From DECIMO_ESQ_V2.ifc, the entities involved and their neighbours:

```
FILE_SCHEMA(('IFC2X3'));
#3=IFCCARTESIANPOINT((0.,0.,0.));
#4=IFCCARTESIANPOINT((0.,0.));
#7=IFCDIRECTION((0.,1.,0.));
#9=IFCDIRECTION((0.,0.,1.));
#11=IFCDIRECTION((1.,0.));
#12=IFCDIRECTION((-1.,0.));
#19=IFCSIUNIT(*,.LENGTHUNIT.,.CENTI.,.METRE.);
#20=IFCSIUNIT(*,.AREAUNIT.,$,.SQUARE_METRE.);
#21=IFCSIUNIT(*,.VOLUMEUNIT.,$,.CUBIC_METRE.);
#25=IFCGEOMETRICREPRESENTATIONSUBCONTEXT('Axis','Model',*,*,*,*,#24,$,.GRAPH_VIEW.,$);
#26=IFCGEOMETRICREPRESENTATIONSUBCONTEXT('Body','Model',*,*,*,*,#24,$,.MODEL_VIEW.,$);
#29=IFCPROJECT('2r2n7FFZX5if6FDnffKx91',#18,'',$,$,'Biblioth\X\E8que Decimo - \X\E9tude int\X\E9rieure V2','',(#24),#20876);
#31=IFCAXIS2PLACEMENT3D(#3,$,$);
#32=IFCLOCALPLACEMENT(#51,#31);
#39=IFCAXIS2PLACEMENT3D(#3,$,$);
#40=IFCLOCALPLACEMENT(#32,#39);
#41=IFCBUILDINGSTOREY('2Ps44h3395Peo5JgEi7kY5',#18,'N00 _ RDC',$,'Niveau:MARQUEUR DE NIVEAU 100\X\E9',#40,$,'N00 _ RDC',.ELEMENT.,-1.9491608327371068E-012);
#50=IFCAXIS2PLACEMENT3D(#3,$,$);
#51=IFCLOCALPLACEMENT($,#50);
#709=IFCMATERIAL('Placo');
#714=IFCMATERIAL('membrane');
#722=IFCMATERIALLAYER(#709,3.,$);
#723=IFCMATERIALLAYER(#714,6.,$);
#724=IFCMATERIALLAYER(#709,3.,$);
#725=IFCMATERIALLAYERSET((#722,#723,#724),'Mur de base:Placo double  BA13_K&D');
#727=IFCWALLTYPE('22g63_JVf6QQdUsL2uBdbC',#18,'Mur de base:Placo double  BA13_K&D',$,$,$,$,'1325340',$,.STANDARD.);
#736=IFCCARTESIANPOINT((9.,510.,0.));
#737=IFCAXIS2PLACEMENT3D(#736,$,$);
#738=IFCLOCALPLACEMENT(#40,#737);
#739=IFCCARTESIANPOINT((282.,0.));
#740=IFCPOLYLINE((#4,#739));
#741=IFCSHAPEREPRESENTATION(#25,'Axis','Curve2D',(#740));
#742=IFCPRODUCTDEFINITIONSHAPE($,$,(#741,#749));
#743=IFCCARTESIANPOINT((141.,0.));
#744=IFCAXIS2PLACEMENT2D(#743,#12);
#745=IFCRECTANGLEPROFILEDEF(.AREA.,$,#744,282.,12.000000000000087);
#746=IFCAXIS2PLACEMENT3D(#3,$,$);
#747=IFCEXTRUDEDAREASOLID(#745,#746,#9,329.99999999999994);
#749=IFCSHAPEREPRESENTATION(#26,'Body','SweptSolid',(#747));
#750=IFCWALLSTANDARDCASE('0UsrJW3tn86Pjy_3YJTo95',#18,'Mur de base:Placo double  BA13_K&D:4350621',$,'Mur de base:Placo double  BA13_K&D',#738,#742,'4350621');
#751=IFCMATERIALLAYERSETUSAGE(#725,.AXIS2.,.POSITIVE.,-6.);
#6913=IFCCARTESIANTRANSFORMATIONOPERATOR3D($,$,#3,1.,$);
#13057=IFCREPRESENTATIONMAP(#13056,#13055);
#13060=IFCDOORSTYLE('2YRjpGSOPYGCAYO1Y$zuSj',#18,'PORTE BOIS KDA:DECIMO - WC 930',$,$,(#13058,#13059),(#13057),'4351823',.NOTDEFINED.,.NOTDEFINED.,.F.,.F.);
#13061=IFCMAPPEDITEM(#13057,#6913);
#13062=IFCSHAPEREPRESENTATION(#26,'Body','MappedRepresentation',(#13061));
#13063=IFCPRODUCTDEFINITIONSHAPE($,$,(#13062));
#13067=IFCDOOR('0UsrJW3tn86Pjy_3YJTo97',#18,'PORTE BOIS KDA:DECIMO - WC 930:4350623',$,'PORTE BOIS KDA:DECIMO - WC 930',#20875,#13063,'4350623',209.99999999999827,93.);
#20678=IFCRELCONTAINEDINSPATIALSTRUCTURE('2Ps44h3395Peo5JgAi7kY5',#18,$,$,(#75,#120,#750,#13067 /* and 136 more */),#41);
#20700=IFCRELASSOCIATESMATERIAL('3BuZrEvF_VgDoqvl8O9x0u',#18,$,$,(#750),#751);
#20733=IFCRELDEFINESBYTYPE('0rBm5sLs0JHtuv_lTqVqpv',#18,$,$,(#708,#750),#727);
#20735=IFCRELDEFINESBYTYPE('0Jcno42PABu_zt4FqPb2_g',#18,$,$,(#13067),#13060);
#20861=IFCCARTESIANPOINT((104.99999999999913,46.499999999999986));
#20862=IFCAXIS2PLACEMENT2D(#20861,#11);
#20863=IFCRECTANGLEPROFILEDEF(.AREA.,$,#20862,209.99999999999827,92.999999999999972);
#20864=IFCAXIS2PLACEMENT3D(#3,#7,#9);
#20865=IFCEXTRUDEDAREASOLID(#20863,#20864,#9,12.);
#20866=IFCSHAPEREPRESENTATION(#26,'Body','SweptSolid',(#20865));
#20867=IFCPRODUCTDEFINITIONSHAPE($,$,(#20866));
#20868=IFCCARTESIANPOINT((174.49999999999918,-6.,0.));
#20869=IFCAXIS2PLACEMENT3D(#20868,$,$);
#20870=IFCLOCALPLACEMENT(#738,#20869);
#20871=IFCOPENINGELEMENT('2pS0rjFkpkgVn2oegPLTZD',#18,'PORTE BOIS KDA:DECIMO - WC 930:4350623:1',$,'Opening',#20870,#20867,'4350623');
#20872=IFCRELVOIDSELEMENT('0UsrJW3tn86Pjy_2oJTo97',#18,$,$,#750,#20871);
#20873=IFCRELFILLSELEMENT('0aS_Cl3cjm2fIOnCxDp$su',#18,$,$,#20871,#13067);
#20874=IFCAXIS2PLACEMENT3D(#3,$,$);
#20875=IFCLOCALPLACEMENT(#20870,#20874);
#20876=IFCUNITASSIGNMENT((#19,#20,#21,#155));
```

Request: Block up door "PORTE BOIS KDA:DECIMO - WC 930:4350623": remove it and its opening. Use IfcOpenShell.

```python
import ifcopenshell
import ifcopenshell.api.feature
import ifcopenshell.api.root
import ifcopenshell.geom
import ifcopenshell.util.shape

model = ifcopenshell.open("DECIMO_ESQ_V2.ifc")
settings = ifcopenshell.geom.settings()


def volume(element):
    """Net volume in cubic metres, openings subtracted."""
    shape = ifcopenshell.geom.create_shape(settings, element)
    return ifcopenshell.util.shape.get_volume(shape.geometry)


door = model.by_guid("0UsrJW3tn86Pjy_3YJTo97")
opening = door.FillsVoids[0].RelatingOpeningElement
wall = opening.VoidsElements[0].RelatingBuildingElement
before = volume(wall)

ifcopenshell.api.root.remove_product(model, product=door)
ifcopenshell.api.feature.remove_feature(model, feature=opening)

after = volume(wall)

print(f"wall volume {before:.3f} -> {after:.3f} m3")

model.write("DECIMO_ESQ_V2_updated.ifc")
```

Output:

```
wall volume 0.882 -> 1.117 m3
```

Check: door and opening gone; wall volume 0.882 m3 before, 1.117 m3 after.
